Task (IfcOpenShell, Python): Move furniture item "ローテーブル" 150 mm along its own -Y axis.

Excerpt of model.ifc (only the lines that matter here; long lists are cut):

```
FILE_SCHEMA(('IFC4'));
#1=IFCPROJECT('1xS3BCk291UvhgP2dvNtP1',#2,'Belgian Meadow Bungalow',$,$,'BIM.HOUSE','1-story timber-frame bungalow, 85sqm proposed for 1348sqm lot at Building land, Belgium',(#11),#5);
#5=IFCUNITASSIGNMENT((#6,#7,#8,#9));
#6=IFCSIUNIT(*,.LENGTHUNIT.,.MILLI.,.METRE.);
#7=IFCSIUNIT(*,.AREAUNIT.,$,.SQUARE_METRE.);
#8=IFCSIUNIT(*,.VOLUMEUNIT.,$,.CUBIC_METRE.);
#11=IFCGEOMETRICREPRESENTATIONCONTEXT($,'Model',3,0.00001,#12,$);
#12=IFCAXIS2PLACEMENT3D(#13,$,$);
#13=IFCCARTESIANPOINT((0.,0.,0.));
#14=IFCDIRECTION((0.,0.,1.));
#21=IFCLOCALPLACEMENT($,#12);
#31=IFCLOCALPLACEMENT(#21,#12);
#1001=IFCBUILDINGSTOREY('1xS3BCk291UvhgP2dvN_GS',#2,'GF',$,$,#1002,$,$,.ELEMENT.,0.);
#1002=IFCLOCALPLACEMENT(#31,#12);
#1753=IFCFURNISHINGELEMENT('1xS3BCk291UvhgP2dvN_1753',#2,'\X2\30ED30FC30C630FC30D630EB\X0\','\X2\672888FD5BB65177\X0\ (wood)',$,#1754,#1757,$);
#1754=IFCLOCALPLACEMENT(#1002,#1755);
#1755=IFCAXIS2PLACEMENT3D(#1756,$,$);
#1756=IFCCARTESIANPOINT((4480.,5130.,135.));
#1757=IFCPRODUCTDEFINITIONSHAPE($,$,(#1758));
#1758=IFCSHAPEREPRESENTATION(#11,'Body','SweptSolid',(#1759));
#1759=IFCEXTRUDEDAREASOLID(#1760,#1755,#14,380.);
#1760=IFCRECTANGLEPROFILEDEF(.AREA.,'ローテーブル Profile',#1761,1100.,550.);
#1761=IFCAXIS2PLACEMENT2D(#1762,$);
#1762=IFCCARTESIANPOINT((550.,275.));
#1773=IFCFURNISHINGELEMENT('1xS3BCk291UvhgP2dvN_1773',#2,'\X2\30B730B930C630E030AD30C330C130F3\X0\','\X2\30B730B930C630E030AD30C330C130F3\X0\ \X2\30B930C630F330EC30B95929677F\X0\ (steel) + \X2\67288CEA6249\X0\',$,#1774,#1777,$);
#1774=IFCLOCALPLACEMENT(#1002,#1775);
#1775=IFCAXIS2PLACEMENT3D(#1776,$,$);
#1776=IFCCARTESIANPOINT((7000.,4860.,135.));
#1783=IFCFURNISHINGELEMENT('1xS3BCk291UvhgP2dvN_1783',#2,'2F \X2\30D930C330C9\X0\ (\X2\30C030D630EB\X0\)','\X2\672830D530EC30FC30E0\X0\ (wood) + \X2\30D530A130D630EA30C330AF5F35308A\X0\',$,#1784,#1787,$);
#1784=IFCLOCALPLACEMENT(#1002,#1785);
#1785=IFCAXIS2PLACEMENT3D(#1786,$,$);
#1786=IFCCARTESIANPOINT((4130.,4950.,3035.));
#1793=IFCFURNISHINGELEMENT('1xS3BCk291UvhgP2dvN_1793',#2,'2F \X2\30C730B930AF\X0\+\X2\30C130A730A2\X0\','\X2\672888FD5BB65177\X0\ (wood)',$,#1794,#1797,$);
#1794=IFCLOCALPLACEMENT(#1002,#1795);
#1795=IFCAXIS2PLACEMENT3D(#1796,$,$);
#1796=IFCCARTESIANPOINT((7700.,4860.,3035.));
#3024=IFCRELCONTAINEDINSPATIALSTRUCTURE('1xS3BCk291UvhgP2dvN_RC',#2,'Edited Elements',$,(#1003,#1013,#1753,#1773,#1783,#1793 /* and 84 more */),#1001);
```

```python
import ifcopenshell
import ifcopenshell.api.geometry
import ifcopenshell.util.placement

model = ifcopenshell.open("model.ifc")

item = model.by_id(1753)
matrix = ifcopenshell.util.placement.get_local_placement(item.ObjectPlacement)
matrix[:3, 3] -= matrix[:3, 1] * 150.0
ifcopenshell.api.geometry.edit_object_placement(model, product=item, matrix=matrix, is_si=False)

print(ifcopenshell.util.placement.get_local_placement(item.ObjectPlacement).round(3) + 0.0)

model.write("model_edited.ifc")
```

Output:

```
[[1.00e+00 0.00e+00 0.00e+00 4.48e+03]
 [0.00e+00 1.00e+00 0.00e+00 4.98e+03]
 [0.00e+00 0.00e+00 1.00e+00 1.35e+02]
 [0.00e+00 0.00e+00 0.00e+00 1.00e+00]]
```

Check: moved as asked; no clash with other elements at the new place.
